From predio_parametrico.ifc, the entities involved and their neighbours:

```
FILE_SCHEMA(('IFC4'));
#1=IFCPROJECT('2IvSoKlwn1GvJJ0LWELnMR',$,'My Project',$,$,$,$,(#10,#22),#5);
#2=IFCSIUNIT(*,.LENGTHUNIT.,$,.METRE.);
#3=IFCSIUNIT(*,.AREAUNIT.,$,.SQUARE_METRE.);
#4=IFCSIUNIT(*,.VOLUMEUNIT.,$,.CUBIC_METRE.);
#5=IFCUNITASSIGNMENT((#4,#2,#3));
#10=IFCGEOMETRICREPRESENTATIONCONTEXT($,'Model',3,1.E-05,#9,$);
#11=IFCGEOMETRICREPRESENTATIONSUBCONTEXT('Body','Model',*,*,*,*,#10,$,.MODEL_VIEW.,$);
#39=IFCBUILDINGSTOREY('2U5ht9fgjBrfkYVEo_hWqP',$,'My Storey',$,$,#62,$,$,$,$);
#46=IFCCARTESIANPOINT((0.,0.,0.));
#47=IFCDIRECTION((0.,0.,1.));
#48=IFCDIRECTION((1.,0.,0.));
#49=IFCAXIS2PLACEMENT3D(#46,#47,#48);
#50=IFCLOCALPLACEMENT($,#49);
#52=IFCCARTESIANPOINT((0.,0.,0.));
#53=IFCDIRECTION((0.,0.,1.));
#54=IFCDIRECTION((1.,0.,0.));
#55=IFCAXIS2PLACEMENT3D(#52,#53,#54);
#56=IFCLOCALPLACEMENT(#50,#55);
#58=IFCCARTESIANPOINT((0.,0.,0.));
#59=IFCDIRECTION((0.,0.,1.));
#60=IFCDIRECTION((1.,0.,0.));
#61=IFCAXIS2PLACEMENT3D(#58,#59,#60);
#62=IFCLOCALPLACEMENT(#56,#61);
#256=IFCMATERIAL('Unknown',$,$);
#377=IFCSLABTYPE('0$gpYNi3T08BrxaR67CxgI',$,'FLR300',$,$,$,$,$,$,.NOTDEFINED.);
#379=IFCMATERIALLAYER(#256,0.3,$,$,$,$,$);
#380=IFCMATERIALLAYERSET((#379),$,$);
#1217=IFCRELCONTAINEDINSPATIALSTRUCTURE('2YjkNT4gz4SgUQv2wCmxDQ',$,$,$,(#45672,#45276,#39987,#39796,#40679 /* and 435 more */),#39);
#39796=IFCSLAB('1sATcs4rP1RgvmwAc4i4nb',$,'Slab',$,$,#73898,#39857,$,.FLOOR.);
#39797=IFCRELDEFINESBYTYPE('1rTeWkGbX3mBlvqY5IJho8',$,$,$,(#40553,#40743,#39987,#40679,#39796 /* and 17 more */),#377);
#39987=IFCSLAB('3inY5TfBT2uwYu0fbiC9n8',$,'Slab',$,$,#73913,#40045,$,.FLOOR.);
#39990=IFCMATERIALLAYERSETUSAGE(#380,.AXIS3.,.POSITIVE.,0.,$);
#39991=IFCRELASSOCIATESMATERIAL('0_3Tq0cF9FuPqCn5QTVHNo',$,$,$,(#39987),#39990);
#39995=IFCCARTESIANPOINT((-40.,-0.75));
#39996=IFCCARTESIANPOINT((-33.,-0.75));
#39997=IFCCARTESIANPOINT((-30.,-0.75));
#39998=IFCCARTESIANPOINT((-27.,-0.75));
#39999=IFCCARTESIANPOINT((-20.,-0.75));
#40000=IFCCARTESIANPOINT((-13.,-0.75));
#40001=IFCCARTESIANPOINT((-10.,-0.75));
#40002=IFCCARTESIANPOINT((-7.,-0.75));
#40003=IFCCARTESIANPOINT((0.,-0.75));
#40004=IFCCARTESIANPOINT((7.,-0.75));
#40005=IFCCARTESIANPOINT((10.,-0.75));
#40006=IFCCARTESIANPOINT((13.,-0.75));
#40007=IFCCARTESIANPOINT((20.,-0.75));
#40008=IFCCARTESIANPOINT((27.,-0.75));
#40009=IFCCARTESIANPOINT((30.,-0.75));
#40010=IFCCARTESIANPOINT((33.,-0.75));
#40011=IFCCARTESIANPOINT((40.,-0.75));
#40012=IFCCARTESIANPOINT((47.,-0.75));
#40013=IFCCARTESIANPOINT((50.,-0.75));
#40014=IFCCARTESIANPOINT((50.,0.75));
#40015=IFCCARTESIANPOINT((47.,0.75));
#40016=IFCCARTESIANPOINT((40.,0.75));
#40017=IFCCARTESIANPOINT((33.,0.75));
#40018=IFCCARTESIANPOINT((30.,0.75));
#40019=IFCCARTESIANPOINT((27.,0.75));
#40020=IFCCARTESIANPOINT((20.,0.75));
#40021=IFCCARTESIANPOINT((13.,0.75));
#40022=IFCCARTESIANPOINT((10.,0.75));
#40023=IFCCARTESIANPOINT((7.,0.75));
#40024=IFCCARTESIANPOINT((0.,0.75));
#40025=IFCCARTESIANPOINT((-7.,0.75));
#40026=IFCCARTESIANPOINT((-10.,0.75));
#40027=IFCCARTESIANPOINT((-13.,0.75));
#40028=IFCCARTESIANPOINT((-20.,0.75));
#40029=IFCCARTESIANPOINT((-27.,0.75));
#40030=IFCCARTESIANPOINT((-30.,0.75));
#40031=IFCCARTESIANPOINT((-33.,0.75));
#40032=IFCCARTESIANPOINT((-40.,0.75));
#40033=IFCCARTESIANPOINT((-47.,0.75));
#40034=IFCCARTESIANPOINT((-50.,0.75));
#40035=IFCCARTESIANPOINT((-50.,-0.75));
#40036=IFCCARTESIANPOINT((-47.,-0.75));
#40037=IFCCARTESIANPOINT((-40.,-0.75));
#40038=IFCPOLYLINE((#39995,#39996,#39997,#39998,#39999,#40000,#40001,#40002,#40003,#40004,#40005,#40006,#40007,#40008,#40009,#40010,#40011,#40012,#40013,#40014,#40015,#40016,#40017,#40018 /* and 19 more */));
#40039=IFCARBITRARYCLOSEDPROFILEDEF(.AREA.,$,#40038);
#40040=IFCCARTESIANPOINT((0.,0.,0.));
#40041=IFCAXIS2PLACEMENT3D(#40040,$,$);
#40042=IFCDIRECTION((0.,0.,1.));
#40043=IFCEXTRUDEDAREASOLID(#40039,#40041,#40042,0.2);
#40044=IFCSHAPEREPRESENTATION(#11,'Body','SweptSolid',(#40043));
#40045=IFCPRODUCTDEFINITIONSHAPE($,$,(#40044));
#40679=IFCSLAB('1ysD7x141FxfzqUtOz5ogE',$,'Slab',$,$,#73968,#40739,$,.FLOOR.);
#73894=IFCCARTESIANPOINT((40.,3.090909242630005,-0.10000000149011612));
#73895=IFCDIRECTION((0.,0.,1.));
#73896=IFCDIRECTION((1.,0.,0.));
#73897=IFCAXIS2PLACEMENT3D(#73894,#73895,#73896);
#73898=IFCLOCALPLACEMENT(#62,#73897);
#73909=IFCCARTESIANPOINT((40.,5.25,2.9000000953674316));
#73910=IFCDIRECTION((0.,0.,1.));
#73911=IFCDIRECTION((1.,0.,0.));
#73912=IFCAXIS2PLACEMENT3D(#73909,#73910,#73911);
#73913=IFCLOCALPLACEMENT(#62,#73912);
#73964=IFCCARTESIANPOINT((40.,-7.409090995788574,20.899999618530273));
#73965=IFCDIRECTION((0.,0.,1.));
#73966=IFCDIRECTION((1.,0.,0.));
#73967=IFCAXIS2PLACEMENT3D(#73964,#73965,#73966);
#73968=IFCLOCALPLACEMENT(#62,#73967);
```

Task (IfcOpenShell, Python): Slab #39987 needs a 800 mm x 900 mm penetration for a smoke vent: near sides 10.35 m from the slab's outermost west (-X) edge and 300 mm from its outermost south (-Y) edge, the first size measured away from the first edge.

```python
import numpy as np
import ifcopenshell
import ifcopenshell.api.feature
import ifcopenshell.api.geometry
import ifcopenshell.api.root
import ifcopenshell.geom
import ifcopenshell.util.placement
import ifcopenshell.util.representation
import ifcopenshell.util.shape
import ifcopenshell.util.unit

model = ifcopenshell.open("predio_parametrico.ifc")
unit_scale = ifcopenshell.util.unit.calculate_unit_scale(model)
settings = ifcopenshell.geom.settings()


def volume(element):
    """Net volume in cubic metres, openings subtracted."""
    shape = ifcopenshell.geom.create_shape(settings, element)
    return ifcopenshell.util.shape.get_volume(shape.geometry)


slab = model.by_guid("3inY5TfBT2uwYu0fbiC9n8")
before = volume(slab)

# Extent in the slab's own axes, in metres. The edges named are its -X and -Y sides.
slab_shape = ifcopenshell.geom.create_shape(settings, slab)
vertices = ifcopenshell.util.shape.get_vertices(slab_shape.geometry)
x_min, y_min, bottom = vertices.min(axis=0)
top = vertices[:, 2].max()

opening = ifcopenshell.api.root.create_entity(model, ifc_class="IfcOpeningElement", name="Smoke vent opening", predefined_type="OPENING")
context = ifcopenshell.util.representation.get_context(model, "Model", "Body", "MODEL_VIEW")
width, depth = 0.8, 0.9
outline = [(0.0, 0.0), (width, 0.0), (width, depth), (0.0, depth), (0.0, 0.0)]
# Overshoot both faces by 50 mm so the cut is clean.
shape = ifcopenshell.api.geometry.add_slab_representation(
    model, context=context, depth=top - bottom + 0.1, polyline=outline
)
ifcopenshell.api.geometry.assign_representation(model, product=opening, representation=shape)

matrix = ifcopenshell.util.placement.get_local_placement(slab.ObjectPlacement)
matrix[:, 3] = matrix @ np.append(np.array([x_min + 10.35, y_min + 0.3, bottom - 0.05]) / unit_scale, 1.0)
ifcopenshell.api.geometry.edit_object_placement(model, product=opening, matrix=matrix, is_si=False)
ifcopenshell.api.feature.add_feature(model, feature=opening, element=slab)

after = volume(slab)

print(f"slab volume {before:.3f} -> {after:.3f} m3")

model.write("predio_parametrico_v2.ifc")
```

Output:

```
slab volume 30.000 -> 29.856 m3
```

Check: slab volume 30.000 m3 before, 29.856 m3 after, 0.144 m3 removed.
